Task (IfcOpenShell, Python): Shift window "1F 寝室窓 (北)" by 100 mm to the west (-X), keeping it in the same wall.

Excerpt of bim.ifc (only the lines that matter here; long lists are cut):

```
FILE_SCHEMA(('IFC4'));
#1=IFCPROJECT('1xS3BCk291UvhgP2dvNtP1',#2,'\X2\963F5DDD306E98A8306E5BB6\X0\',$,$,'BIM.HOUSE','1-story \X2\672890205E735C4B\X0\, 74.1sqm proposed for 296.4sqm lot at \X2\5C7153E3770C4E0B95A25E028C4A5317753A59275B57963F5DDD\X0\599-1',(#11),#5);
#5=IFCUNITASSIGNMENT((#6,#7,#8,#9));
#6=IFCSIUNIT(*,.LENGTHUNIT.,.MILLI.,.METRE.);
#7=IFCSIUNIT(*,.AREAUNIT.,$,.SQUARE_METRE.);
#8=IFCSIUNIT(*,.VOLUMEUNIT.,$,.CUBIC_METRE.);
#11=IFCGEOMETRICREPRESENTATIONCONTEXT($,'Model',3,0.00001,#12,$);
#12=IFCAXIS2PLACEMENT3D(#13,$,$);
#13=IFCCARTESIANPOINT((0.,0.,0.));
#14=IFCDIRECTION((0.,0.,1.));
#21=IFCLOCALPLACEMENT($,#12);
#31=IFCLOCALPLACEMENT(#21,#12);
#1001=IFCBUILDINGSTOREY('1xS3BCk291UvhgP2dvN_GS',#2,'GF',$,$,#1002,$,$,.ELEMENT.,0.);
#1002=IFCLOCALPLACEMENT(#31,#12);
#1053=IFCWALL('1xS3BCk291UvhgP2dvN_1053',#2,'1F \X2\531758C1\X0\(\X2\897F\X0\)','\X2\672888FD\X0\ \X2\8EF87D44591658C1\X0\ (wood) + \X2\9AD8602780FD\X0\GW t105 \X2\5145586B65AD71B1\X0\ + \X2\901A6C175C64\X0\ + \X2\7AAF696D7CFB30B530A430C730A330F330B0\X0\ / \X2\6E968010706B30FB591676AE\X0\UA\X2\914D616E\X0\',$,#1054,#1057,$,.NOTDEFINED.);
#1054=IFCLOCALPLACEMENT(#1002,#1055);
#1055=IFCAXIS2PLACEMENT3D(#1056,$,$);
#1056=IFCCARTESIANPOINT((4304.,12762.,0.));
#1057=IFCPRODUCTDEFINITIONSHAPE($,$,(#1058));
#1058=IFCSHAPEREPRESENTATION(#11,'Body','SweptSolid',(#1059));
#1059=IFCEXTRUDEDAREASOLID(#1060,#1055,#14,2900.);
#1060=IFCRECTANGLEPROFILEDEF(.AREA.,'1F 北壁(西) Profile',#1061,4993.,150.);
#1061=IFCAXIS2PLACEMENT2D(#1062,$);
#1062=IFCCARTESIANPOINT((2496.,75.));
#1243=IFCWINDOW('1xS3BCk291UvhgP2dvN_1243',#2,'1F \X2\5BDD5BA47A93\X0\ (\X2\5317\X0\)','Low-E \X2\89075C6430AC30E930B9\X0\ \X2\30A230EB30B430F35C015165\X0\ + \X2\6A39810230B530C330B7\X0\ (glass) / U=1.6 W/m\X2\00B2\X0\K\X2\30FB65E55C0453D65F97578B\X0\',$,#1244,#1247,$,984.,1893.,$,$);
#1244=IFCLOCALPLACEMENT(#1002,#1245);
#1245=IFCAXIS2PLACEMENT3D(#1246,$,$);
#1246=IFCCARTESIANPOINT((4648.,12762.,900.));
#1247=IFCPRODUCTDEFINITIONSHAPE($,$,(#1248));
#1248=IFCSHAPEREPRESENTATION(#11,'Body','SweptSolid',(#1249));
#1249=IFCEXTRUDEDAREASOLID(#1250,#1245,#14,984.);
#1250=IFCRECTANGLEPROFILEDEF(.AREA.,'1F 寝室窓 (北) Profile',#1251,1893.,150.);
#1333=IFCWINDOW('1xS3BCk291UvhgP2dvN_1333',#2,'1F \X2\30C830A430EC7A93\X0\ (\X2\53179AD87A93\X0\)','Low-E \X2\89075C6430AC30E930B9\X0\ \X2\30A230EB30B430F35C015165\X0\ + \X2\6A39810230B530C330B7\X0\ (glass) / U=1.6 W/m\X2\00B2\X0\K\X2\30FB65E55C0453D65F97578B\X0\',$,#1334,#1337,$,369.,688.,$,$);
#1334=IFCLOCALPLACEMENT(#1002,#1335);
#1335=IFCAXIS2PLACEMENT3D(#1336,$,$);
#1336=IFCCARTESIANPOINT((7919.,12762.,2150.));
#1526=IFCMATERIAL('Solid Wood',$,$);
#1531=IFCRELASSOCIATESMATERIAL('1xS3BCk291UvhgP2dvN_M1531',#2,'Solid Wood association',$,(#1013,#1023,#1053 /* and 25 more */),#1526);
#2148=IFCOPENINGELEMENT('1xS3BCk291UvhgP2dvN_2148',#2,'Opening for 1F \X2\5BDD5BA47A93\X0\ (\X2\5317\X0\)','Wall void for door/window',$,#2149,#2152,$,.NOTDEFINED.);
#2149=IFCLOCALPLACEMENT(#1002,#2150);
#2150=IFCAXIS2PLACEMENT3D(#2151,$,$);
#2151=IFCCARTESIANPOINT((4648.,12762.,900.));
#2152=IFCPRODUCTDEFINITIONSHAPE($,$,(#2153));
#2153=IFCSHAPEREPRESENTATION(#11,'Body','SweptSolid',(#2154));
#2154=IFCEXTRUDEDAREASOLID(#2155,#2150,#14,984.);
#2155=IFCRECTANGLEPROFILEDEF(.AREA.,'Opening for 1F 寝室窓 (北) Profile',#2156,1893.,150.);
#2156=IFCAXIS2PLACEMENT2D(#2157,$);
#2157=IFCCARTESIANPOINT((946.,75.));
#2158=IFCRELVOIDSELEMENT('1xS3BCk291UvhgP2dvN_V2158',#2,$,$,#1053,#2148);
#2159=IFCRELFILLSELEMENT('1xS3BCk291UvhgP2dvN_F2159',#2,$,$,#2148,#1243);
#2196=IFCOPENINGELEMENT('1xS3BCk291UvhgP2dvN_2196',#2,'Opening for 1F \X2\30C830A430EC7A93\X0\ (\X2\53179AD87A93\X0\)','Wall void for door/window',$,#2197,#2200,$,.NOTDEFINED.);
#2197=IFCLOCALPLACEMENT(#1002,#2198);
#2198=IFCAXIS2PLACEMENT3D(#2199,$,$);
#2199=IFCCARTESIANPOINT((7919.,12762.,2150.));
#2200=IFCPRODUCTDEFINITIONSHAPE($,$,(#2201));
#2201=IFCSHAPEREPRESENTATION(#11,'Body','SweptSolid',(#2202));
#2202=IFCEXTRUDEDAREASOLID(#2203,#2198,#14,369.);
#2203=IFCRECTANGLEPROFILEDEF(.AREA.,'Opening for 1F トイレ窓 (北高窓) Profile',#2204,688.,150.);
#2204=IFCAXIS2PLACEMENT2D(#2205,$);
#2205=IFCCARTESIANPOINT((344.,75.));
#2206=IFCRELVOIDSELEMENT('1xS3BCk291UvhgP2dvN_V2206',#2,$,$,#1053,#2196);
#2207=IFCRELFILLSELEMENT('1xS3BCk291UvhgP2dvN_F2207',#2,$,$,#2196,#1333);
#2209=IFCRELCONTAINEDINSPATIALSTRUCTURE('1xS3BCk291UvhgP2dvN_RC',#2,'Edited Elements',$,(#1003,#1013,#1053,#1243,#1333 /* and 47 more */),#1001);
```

```python
import ifcopenshell
import ifcopenshell.api.geometry
import ifcopenshell.util.placement

model = ifcopenshell.open("bim.ifc")

window = model.by_guid("1xS3BCk291UvhgP2dvN_1243")
opening = window.FillsVoids[0].RelatingOpeningElement
wall = opening.VoidsElements[0].RelatingBuildingElement

wall_matrix = ifcopenshell.util.placement.get_local_placement(wall.ObjectPlacement)
shift = wall_matrix[:3, 0] * -100.0
before = ifcopenshell.util.placement.get_local_placement(window.ObjectPlacement)[:3, 3].copy()

# The window is not placed relative to its opening, so move both.
for product in (opening, window):
    matrix = ifcopenshell.util.placement.get_local_placement(product.ObjectPlacement)
    matrix[:3, 3] += shift
    ifcopenshell.api.geometry.edit_object_placement(model, product=product, matrix=matrix, is_si=False)

after = ifcopenshell.util.placement.get_local_placement(window.ObjectPlacement)[:3, 3]
print("window moved by", (after - before).round(3) + 0.0)

model.write("bim_rev.ifc")
```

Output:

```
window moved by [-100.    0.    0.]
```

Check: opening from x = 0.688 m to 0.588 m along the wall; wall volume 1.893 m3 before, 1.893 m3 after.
